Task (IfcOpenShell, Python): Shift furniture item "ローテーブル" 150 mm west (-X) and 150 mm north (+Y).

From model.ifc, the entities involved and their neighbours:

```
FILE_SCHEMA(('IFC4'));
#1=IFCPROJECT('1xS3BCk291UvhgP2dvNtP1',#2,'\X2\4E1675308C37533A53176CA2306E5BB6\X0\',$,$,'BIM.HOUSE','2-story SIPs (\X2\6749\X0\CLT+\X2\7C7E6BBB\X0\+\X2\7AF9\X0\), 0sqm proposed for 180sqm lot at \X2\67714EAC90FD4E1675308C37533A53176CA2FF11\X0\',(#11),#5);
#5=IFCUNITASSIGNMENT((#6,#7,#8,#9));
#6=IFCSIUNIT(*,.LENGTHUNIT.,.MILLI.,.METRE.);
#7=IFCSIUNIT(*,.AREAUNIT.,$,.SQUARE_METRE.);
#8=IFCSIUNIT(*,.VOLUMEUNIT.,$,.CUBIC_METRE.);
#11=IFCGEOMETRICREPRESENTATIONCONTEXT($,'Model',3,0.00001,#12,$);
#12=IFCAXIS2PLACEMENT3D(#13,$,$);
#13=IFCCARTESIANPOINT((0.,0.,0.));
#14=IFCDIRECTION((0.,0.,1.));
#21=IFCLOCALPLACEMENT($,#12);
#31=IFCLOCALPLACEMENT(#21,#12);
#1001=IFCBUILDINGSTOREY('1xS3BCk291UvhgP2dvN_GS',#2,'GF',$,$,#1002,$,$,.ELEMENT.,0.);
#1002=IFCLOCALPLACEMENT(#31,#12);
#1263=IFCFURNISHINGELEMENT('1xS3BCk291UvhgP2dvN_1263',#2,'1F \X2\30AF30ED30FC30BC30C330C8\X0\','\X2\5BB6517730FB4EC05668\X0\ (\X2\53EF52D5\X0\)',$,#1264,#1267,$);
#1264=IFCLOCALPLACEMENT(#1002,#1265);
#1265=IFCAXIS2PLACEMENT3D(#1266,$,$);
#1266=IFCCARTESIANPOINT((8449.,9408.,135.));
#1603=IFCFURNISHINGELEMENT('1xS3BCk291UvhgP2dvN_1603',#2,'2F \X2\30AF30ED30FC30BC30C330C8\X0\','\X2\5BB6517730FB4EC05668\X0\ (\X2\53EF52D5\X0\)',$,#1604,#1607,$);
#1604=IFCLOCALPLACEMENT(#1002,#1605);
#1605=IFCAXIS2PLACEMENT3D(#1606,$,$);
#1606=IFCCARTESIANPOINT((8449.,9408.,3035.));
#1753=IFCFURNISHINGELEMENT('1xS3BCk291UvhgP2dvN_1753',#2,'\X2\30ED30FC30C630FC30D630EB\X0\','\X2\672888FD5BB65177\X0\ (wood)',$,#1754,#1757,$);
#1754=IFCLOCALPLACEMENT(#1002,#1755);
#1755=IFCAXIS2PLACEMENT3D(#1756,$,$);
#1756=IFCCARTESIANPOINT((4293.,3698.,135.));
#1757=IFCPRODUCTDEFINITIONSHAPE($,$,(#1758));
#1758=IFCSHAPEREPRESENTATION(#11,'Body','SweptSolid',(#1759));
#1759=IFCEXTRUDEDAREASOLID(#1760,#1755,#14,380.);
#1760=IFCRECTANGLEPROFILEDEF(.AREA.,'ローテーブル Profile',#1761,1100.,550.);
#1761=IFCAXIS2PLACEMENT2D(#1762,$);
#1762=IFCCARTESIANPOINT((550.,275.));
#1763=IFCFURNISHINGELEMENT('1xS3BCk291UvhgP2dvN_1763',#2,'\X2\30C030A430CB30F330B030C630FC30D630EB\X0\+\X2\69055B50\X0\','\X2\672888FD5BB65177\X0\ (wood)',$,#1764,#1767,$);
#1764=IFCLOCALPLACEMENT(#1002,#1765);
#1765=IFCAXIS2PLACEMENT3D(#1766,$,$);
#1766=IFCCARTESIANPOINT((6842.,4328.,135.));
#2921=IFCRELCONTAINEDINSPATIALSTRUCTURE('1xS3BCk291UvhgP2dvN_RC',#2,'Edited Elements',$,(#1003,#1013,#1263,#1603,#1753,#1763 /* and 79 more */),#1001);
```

```python
import ifcopenshell
import ifcopenshell.api.geometry
import ifcopenshell.util.placement

model = ifcopenshell.open("model.ifc")

item = model.by_guid("1xS3BCk291UvhgP2dvN_1753")
matrix = ifcopenshell.util.placement.get_local_placement(item.ObjectPlacement)
matrix[0, 3] -= 150.0
matrix[1, 3] += 150.0
ifcopenshell.api.geometry.edit_object_placement(model, product=item, matrix=matrix, is_si=False)

print(ifcopenshell.util.placement.get_local_placement(item.ObjectPlacement).round(3) + 0.0)

model.write("model_updated.ifc")
```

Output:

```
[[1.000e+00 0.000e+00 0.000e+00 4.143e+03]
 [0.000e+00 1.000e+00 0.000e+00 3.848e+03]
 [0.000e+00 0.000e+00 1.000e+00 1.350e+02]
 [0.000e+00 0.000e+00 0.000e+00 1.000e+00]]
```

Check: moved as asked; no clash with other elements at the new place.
